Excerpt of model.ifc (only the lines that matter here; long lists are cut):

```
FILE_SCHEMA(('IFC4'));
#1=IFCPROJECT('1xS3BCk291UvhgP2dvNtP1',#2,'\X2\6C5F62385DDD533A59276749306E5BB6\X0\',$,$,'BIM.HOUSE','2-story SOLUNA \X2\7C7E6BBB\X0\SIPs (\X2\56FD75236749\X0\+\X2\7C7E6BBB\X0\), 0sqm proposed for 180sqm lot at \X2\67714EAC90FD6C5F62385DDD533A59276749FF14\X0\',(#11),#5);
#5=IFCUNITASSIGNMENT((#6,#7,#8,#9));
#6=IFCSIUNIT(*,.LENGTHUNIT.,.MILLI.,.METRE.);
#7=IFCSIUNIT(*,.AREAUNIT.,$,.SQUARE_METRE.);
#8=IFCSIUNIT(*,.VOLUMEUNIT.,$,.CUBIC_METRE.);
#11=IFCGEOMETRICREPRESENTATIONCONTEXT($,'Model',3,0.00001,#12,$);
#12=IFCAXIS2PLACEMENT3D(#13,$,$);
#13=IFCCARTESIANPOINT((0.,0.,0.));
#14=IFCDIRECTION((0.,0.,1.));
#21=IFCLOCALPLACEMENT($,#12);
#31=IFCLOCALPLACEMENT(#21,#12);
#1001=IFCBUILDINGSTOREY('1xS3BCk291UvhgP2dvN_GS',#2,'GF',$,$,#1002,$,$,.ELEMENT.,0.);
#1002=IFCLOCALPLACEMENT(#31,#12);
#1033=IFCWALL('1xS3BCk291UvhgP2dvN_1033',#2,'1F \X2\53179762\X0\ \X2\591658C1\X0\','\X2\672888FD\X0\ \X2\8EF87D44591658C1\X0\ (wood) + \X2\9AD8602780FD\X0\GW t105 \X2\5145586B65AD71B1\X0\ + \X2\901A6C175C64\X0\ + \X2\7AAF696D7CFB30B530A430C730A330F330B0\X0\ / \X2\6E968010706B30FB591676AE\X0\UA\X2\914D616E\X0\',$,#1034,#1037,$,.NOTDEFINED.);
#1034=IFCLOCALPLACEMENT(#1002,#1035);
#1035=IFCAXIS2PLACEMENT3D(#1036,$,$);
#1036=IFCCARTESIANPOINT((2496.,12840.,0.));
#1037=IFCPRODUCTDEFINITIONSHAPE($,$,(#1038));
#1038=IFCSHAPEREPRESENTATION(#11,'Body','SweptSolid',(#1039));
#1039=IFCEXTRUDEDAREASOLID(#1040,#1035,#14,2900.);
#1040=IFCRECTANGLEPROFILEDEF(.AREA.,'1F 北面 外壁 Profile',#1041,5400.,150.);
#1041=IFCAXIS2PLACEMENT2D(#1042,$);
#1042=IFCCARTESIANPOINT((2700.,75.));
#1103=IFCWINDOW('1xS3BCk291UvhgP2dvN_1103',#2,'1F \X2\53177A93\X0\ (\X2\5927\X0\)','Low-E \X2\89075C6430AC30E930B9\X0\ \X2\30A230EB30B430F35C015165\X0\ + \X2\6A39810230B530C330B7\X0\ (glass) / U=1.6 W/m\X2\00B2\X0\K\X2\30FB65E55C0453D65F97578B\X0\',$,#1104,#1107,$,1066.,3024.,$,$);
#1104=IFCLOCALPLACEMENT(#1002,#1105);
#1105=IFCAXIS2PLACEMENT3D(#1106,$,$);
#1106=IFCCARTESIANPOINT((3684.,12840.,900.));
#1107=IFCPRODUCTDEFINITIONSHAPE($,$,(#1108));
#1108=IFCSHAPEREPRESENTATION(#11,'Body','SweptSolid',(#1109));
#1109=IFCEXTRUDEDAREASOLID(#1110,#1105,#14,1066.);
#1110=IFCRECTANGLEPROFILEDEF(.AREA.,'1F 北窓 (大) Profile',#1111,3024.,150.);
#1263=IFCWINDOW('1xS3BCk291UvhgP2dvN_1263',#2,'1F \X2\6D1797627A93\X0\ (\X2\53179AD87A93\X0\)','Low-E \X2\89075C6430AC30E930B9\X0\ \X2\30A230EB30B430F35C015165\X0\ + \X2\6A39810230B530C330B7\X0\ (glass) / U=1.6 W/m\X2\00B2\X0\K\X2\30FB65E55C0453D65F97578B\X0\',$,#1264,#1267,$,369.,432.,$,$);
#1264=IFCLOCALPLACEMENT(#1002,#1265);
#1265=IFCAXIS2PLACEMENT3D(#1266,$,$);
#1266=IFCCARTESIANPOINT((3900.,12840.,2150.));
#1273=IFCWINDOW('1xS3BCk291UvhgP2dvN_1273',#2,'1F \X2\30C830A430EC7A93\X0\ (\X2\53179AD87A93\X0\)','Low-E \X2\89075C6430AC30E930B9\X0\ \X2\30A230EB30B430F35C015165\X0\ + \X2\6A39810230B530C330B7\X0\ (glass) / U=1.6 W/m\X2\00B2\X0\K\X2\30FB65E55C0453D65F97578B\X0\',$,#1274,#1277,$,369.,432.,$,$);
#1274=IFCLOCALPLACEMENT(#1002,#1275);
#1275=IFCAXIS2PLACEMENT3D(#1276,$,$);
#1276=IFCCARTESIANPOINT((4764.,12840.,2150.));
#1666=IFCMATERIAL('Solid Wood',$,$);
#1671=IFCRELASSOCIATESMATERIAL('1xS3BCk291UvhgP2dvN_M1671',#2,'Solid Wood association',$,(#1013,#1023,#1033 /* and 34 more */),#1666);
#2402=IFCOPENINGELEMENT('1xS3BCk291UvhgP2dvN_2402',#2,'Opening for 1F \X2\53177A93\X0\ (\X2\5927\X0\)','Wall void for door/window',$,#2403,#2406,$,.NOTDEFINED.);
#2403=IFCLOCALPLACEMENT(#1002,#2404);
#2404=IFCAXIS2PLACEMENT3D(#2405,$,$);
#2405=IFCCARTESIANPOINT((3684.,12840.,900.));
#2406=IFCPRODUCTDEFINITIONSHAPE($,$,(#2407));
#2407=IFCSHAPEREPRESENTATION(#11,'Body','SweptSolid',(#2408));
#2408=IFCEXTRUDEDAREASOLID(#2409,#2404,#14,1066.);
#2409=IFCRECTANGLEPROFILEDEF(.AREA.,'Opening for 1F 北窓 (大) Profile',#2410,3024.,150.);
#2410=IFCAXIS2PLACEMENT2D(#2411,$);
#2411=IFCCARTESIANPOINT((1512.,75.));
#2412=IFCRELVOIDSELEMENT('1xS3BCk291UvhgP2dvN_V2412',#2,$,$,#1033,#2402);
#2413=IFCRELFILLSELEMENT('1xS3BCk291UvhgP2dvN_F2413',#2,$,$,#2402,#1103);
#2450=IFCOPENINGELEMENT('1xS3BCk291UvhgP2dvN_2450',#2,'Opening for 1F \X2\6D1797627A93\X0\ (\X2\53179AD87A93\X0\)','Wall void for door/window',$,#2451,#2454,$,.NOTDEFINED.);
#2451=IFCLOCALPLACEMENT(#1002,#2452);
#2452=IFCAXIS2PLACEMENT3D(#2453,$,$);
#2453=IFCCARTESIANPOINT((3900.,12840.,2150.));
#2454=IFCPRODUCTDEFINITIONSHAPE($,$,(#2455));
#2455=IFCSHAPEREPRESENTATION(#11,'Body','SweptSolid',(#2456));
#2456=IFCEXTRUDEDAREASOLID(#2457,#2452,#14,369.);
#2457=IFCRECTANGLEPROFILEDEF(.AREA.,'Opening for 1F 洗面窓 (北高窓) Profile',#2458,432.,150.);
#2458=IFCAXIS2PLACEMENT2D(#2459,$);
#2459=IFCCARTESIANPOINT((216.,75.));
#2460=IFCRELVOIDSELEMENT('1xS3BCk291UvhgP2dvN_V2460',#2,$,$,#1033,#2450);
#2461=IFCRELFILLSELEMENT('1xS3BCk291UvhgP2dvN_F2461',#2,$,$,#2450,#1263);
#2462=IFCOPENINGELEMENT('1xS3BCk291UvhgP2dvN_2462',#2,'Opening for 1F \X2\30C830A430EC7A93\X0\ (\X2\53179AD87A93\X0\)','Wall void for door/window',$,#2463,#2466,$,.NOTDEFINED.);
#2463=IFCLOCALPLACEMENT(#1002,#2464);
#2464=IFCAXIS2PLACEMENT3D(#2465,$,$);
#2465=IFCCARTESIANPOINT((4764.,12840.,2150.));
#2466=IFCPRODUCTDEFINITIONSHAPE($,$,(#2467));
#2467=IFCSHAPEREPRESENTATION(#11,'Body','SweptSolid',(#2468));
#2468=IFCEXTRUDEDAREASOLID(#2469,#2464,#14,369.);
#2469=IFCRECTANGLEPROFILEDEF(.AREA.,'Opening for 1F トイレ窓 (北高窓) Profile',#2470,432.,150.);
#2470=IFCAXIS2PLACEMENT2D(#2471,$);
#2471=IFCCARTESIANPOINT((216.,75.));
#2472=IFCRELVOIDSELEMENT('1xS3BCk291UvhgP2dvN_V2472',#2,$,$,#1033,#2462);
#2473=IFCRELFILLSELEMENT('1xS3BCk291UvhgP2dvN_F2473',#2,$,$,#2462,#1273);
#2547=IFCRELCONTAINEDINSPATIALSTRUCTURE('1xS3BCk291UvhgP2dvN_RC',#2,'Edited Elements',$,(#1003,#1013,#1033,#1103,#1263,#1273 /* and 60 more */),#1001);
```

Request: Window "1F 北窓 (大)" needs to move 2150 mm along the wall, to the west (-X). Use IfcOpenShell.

```python
import ifcopenshell
import ifcopenshell.api.geometry
import ifcopenshell.util.placement
import ifcopenshell.util.unit

model = ifcopenshell.open("model.ifc")
unit_scale = ifcopenshell.util.unit.calculate_unit_scale(model)

window = model.by_guid("1xS3BCk291UvhgP2dvN_1103")
opening = window.FillsVoids[0].RelatingOpeningElement
wall = opening.VoidsElements[0].RelatingBuildingElement

wall_matrix = ifcopenshell.util.placement.get_local_placement(wall.ObjectPlacement)
shift = wall_matrix[:3, 0] * -2.15 / unit_scale
before = ifcopenshell.util.placement.get_local_placement(window.ObjectPlacement)[:3, 3].copy()

# The window is not placed relative to its opening, so move both.
for product in (opening, window):
    matrix = ifcopenshell.util.placement.get_local_placement(product.ObjectPlacement)
    matrix[:3, 3] += shift
    ifcopenshell.api.geometry.edit_object_placement(model, product=product, matrix=matrix, is_si=False)

after = ifcopenshell.util.placement.get_local_placement(window.ObjectPlacement)[:3, 3]
print("window moved by", (after - before).round(3) + 0.0)

model.write("model-out.ifc")
```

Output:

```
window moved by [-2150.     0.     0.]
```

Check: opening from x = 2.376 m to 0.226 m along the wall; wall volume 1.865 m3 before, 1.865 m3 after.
